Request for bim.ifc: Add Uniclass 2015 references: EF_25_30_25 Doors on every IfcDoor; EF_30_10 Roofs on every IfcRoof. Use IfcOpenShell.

First a look at what the model holds.

```python
import ifcopenshell

model = ifcopenshell.open("bim.ifc")
print(model.schema)
print("classifications:", [c.Name for c in model.by_type("IfcClassification")])
for ifc_class in ("IfcDoor", "IfcRoof", "IfcStair", "IfcWall", "IfcWindow"):
    print(ifc_class, len(model.by_type(ifc_class)))
```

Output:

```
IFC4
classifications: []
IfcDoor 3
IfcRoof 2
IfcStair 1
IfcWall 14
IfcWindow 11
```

```python
import ifcopenshell
import ifcopenshell.api.classification

model = ifcopenshell.open("bim.ifc")

system = ifcopenshell.api.classification.add_classification(model, classification="Uniclass 2015")

codes = {
    "IfcDoor": ("EF_25_30_25", "Doors"),
    "IfcRoof": ("EF_30_10", "Roofs"),
}
for ifc_class, (code, name) in codes.items():
    products = model.by_type(ifc_class)
    ifcopenshell.api.classification.add_reference(
        model, products=products, classification=system, identification=code, name=name
    )
    print(code, len(products))

model.write("bim_v2.ifc")
```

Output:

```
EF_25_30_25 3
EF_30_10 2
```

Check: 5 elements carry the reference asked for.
